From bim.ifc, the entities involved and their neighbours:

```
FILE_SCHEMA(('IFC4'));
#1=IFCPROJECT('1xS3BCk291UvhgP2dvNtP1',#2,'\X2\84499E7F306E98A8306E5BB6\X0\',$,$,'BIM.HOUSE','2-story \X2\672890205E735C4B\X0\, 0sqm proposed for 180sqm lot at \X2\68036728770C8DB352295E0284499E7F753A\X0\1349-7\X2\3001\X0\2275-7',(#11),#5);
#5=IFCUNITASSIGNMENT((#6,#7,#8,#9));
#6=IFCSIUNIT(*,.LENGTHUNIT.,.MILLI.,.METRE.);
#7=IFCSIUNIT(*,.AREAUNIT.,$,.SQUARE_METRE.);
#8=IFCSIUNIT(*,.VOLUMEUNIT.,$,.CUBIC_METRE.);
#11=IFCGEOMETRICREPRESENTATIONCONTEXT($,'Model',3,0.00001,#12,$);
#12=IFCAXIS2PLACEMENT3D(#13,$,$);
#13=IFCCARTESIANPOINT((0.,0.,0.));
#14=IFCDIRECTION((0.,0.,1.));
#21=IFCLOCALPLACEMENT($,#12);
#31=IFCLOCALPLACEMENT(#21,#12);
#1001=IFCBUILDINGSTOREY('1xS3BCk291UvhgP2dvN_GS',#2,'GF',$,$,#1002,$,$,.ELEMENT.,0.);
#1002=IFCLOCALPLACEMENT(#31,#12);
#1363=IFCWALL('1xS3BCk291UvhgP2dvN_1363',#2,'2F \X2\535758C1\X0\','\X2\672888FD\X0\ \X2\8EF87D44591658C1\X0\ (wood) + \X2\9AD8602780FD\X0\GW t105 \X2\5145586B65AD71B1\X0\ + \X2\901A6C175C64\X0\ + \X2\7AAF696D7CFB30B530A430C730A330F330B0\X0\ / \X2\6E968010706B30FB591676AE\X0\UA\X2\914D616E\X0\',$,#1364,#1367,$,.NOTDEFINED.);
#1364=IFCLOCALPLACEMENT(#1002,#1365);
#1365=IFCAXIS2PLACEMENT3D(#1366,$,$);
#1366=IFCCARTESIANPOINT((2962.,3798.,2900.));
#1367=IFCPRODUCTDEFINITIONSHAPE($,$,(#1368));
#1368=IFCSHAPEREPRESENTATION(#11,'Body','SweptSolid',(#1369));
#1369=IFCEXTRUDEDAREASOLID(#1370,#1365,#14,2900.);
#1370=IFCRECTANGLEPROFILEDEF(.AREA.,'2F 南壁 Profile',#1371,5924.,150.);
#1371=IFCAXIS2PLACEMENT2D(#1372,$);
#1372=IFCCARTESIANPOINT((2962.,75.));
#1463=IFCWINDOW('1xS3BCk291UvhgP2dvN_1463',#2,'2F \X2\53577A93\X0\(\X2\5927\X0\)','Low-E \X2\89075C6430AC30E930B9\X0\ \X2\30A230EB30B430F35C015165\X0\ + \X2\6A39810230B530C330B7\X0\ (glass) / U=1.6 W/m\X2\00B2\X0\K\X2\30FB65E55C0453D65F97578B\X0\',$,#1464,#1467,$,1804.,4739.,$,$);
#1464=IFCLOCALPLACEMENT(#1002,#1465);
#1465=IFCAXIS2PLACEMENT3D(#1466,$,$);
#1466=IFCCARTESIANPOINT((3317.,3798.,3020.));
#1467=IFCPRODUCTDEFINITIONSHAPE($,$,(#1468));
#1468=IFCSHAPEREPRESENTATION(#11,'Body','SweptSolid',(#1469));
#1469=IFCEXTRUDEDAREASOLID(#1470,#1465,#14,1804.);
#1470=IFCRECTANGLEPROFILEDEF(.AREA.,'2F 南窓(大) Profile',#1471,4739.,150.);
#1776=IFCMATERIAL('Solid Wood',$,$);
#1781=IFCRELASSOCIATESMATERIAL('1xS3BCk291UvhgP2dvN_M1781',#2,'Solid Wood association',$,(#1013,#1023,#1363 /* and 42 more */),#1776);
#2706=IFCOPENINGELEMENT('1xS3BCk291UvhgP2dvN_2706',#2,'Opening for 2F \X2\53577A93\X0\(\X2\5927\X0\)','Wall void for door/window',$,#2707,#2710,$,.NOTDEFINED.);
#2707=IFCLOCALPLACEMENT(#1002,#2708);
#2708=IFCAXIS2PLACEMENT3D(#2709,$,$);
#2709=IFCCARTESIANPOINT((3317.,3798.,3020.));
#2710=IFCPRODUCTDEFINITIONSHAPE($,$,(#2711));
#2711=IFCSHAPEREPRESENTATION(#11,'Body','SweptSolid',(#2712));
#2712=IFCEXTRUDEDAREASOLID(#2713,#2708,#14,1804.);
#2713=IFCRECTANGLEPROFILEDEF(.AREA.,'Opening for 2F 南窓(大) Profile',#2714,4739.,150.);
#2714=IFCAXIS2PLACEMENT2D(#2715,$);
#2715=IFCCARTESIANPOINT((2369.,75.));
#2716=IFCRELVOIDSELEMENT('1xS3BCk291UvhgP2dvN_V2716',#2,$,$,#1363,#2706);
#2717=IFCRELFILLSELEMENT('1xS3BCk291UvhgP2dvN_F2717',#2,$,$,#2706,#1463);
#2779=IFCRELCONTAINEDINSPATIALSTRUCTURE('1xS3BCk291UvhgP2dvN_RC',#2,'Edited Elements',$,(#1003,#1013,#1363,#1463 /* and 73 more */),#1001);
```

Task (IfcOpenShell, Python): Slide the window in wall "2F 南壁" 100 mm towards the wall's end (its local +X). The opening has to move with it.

```python
import ifcopenshell
import ifcopenshell.api.geometry
import ifcopenshell.util.placement
import ifcopenshell.util.unit

model = ifcopenshell.open("bim.ifc")
unit_scale = ifcopenshell.util.unit.calculate_unit_scale(model)

window = model.by_guid("1xS3BCk291UvhgP2dvN_1463")
opening = window.FillsVoids[0].RelatingOpeningElement
wall = opening.VoidsElements[0].RelatingBuildingElement

wall_matrix = ifcopenshell.util.placement.get_local_placement(wall.ObjectPlacement)
shift = wall_matrix[:3, 0] * 0.1 / unit_scale
before = ifcopenshell.util.placement.get_local_placement(window.ObjectPlacement)[:3, 3].copy()

# The window is not placed relative to its opening, so move both.
for product in (opening, window):
    matrix = ifcopenshell.util.placement.get_local_placement(product.ObjectPlacement)
    matrix[:3, 3] += shift
    ifcopenshell.api.geometry.edit_object_placement(model, product=product, matrix=matrix, is_si=False)

after = ifcopenshell.util.placement.get_local_placement(window.ObjectPlacement)[:3, 3]
print("window moved by", (after - before).round(3) + 0.0)

model.write("bim_rev.ifc")
```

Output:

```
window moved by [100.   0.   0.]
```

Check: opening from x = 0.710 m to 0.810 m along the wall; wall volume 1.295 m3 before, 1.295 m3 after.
